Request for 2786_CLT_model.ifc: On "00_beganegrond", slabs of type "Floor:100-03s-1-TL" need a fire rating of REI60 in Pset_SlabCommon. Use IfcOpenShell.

First a look at what the model holds.

```python
import ifcopenshell
import ifcopenshell.util.element

model = ifcopenshell.open("2786_CLT_model.ifc")
print(model.schema)
storey = next(s for s in model.by_type("IfcBuildingStorey") if s.Name == "00_beganegrond")
slabs = [e for e in ifcopenshell.util.element.get_decomposition(storey) if e.is_a("IfcSlab")]
seen = {}
for e in slabs:
    element_type = ifcopenshell.util.element.get_type(e)
    key = (element_type.Name if element_type != e and element_type else None, ifcopenshell.util.element.get_pset(e, "Pset_SlabCommon", "FireRating"))
    seen[key] = seen.get(key, 0) + 1
for (name, value), count in sorted(seen.items(), key=str):
    print(count, "x", name, "|", value)
```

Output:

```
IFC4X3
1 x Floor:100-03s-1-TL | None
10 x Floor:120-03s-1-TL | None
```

```python
import ifcopenshell
import ifcopenshell.api.pset
import ifcopenshell.util.element

model = ifcopenshell.open("2786_CLT_model.ifc")

storey = next(s for s in model.by_type("IfcBuildingStorey") if s.Name == "00_beganegrond")
slabs = [e for e in ifcopenshell.util.element.get_decomposition(storey) if e.is_a("IfcSlab")]

count = 0
for e in slabs:
    element_type = ifcopenshell.util.element.get_type(e)
    if element_type in (None, e) or element_type.Name != "Floor:100-03s-1-TL":
        continue
    # add_pset returns the element's existing set when there is one.
    pset = ifcopenshell.api.pset.add_pset(model, product=e, name="Pset_SlabCommon")
    ifcopenshell.api.pset.edit_pset(model, pset=pset, properties={"FireRating": "REI60"})
    count += 1

print(count, "slabs updated")

model.write("2786_CLT_model_updated.ifc")
```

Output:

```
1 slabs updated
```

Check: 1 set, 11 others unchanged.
